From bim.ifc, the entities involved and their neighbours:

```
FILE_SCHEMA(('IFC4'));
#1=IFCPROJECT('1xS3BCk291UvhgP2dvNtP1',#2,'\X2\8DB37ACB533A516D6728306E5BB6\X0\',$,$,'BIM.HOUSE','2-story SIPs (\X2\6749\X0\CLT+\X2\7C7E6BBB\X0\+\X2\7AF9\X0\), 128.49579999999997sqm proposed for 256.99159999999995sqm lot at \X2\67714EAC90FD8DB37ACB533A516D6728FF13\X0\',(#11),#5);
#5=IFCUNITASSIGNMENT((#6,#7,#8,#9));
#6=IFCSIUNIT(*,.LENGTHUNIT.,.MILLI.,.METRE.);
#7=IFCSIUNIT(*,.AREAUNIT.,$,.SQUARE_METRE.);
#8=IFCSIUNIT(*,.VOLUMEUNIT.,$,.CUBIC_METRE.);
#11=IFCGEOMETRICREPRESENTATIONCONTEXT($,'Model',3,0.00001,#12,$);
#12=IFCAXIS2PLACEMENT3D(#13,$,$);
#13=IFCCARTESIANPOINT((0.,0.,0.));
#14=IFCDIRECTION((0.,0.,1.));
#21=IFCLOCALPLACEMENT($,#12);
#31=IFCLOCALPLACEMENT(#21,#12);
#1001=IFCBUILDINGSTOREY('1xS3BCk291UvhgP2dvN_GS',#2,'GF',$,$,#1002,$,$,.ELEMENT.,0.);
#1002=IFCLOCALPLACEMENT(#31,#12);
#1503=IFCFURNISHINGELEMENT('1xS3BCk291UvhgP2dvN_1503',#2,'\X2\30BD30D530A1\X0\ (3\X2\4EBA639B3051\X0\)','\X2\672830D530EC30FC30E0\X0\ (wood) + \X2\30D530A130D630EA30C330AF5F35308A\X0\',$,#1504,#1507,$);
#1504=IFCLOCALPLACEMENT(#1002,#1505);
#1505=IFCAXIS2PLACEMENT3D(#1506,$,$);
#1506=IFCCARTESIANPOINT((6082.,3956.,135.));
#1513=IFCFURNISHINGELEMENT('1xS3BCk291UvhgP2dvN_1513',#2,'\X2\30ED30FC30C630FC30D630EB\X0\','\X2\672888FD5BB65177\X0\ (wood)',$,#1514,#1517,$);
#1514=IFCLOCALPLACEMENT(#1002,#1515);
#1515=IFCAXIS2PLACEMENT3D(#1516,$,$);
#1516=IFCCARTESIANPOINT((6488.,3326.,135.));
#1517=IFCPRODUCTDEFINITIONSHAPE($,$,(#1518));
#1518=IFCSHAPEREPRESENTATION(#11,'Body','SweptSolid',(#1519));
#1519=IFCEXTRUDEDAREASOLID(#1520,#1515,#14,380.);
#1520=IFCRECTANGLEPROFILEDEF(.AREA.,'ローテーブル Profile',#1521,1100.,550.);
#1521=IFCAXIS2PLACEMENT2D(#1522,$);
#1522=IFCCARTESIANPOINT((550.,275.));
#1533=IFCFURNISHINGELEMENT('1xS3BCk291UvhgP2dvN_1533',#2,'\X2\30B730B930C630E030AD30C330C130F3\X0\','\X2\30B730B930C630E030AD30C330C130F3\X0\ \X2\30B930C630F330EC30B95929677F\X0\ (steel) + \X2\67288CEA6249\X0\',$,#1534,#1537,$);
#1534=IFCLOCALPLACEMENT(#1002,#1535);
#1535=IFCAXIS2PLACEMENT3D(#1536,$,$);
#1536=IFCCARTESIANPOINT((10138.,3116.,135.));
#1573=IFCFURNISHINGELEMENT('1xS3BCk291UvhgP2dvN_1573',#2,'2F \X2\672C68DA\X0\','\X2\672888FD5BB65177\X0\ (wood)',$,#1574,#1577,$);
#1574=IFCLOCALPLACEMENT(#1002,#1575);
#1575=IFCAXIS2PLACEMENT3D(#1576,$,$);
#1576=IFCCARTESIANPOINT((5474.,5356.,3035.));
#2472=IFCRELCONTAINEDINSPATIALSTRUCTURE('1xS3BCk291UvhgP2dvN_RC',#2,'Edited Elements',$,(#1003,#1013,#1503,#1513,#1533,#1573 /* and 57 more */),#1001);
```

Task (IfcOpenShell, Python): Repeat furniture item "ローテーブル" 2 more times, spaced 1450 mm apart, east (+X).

```python
import numpy as np
import ifcopenshell
import ifcopenshell.api.geometry
import ifcopenshell.api.root
import ifcopenshell.util.element
import ifcopenshell.util.placement

model = ifcopenshell.open("bim.ifc")


def reuse_history(source, copy):
    """copy_class also copies each property set's owner history, people and application; keep the originals."""
    for rel in copy.IsDefinedBy:
        if rel.is_a("IfcRelDefinesByProperties") and (history := rel.RelatingPropertyDefinition.OwnerHistory):
            rel.RelatingPropertyDefinition.OwnerHistory = source.OwnerHistory
            ifcopenshell.util.element.remove_deep2(model, history)


source = model.by_id(1513)
base = ifcopenshell.util.placement.get_local_placement(source.ObjectPlacement)
step = np.array([1.0, 0.0, 0.0]) * 1450.0

for i in range(1, 3):
    copy = ifcopenshell.api.root.copy_class(model, product=source)
    copy.Representation = ifcopenshell.util.element.copy_deep(
        model, source.Representation, exclude=["IfcGeometricRepresentationContext", "IfcRepresentationMap"]
    )
    reuse_history(source, copy)
    matrix = base.copy()
    matrix[:3, 3] += i * step
    print("added at", matrix[:3, 3].round(3) + 0.0)
    ifcopenshell.api.geometry.edit_object_placement(model, product=copy, matrix=matrix, is_si=False)

model.write("bim_rev.ifc")
```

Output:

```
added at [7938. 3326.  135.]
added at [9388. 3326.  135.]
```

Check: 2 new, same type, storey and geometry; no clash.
